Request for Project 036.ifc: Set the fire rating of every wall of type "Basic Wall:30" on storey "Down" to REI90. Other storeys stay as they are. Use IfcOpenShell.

First a look at what the model holds.

```python
import ifcopenshell
import ifcopenshell.util.element

model = ifcopenshell.open("Project 036.ifc")
print(model.schema)
storey = next(s for s in model.by_type("IfcBuildingStorey") if s.Name == "Down")
walls = [e for e in ifcopenshell.util.element.get_decomposition(storey) if e.is_a("IfcWall")]
seen = {}
for e in walls:
    element_type = ifcopenshell.util.element.get_type(e)
    key = (element_type.Name if element_type != e and element_type else None, ifcopenshell.util.element.get_pset(e, "Pset_WallCommon", "FireRating"))
    seen[key] = seen.get(key, 0) + 1
for (name, value), count in sorted(seen.items(), key=str):
    print(count, "x", name, "|", value)
```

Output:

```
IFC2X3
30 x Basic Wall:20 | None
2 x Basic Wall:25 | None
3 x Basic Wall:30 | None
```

```python
import ifcopenshell
import ifcopenshell.api.pset
import ifcopenshell.util.element

model = ifcopenshell.open("Project 036.ifc")

storey = next(s for s in model.by_type("IfcBuildingStorey") if s.Name == "Down")
walls = [e for e in ifcopenshell.util.element.get_decomposition(storey) if e.is_a("IfcWall")]

count = 0
for e in walls:
    element_type = ifcopenshell.util.element.get_type(e)
    if element_type in (None, e) or element_type.Name != "Basic Wall:30":
        continue
    # add_pset returns the element's existing set when there is one.
    pset = ifcopenshell.api.pset.add_pset(model, product=e, name="Pset_WallCommon")
    ifcopenshell.api.pset.edit_pset(model, pset=pset, properties={"FireRating": "REI90"})
    count += 1

print(count, "walls updated")

model.write("Project 036_edited.ifc")
```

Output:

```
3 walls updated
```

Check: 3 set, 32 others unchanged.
